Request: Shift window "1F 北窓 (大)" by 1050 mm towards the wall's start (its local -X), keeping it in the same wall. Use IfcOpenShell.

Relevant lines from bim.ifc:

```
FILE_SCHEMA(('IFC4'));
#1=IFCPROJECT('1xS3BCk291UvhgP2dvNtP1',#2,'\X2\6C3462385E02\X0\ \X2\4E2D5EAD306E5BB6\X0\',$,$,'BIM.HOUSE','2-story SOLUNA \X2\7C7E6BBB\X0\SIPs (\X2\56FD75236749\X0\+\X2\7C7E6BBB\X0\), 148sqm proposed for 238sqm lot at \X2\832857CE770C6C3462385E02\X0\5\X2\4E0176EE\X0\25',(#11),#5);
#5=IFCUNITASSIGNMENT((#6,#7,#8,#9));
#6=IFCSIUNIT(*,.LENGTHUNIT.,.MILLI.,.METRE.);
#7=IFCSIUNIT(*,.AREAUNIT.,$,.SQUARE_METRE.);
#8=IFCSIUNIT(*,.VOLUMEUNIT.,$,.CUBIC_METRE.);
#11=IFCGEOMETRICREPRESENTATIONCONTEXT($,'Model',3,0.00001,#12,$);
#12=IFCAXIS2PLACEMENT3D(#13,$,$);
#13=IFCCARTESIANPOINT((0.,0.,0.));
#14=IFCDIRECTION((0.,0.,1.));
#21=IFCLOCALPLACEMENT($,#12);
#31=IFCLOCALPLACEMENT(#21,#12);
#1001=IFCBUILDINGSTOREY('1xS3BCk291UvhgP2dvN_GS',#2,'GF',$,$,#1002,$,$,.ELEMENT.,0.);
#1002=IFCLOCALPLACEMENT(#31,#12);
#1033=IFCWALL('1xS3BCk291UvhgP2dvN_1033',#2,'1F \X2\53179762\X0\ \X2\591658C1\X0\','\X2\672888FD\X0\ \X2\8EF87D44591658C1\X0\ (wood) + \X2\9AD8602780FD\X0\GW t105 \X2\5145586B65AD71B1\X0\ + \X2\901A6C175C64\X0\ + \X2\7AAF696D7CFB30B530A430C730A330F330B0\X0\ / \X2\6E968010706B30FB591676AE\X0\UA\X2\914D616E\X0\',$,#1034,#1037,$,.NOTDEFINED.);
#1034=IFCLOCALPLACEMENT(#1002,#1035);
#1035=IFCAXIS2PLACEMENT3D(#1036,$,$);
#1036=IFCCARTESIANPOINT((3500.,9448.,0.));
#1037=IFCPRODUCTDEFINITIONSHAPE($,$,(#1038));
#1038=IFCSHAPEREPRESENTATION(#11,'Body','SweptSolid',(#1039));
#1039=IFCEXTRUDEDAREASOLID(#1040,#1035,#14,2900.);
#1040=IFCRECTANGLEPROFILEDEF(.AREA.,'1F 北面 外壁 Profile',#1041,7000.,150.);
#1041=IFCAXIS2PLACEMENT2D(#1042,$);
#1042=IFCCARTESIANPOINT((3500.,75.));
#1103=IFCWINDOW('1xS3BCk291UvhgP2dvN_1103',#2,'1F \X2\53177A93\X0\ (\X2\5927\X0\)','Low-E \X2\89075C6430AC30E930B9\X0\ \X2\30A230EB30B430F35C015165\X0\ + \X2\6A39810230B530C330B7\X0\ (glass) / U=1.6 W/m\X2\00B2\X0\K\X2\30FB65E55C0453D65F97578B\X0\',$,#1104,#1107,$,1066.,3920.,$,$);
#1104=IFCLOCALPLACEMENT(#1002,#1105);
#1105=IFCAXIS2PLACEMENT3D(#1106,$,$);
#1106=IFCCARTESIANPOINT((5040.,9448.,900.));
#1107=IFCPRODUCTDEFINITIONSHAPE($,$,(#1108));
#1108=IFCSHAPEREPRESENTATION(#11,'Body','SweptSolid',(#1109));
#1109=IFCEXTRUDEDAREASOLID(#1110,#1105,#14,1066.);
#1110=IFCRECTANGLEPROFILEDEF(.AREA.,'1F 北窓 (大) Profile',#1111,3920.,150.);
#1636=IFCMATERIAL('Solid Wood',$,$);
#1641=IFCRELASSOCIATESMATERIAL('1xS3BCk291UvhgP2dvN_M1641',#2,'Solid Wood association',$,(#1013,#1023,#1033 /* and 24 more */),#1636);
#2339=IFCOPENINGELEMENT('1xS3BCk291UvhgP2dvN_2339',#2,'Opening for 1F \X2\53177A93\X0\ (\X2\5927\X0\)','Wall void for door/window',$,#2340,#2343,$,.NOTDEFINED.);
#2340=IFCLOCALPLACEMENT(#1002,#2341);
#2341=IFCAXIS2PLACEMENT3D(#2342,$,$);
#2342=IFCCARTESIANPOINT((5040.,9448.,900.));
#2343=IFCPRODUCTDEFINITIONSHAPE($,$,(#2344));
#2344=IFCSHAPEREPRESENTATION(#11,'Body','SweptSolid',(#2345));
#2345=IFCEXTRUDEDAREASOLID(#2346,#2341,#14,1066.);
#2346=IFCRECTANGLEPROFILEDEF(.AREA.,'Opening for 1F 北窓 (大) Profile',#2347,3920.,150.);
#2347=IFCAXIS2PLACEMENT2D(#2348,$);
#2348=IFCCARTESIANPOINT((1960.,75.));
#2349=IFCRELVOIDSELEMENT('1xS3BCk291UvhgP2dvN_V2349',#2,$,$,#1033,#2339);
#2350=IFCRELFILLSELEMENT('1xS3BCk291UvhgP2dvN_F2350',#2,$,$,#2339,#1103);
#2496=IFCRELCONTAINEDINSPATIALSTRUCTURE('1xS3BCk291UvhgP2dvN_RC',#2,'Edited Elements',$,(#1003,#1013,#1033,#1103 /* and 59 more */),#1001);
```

```python
import ifcopenshell
import ifcopenshell.api.geometry
import ifcopenshell.util.placement

model = ifcopenshell.open("bim.ifc")

window = model.by_guid("1xS3BCk291UvhgP2dvN_1103")
opening = window.FillsVoids[0].RelatingOpeningElement
wall = opening.VoidsElements[0].RelatingBuildingElement

wall_matrix = ifcopenshell.util.placement.get_local_placement(wall.ObjectPlacement)
shift = wall_matrix[:3, 0] * -1050.0
before = ifcopenshell.util.placement.get_local_placement(window.ObjectPlacement)[:3, 3].copy()

# The window is not placed relative to its opening, so move both.
for product in (opening, window):
    matrix = ifcopenshell.util.placement.get_local_placement(product.ObjectPlacement)
    matrix[:3, 3] += shift
    ifcopenshell.api.geometry.edit_object_placement(model, product=product, matrix=matrix, is_si=False)

after = ifcopenshell.util.placement.get_local_placement(window.ObjectPlacement)[:3, 3]
print("window moved by", (after - before).round(3) + 0.0)

model.write("bim_v2.ifc")
```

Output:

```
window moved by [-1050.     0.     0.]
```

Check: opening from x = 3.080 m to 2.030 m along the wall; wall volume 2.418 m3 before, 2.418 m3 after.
